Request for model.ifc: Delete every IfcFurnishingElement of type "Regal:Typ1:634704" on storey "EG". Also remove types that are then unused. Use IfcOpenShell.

First a look at what the model holds.

```python
import ifcopenshell
import ifcopenshell.util.element

model = ifcopenshell.open("model.ifc")
print(model.schema)
storey = next(s for s in model.by_type("IfcBuildingStorey") if s.Name == "EG")
furniture = [e for e in ifcopenshell.util.element.get_decomposition(storey) if e.is_a("IfcFurnishingElement")]
seen = {}
for e in furniture:
    element_type = ifcopenshell.util.element.get_type(e)
    name = element_type.Name if element_type not in (None, e) else None
    seen[name] = seen.get(name, 0) + 1
for name, count in sorted(seen.items(), key=str):
    print(count, "x", name)
```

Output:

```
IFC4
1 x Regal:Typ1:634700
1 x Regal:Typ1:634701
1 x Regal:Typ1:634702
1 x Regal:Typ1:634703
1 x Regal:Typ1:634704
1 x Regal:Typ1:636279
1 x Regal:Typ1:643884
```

```python
import ifcopenshell
import ifcopenshell.api.root
import ifcopenshell.util.element

model = ifcopenshell.open("model.ifc")

storey = next(s for s in model.by_type("IfcBuildingStorey") if s.Name == "EG")
furniture = [e for e in ifcopenshell.util.element.get_decomposition(storey) if e.is_a("IfcFurnishingElement")]
targets = [e for e in furniture if (t := ifcopenshell.util.element.get_type(e)) not in (None, e) and t.Name == "Regal:Typ1:634704"]
types = {ifcopenshell.util.element.get_type(e) for e in targets} - {None, *targets}

for e in targets:
    ifcopenshell.api.root.remove_product(model, product=e)
print(len(targets), "removed")

unused = [t for t in types if not ifcopenshell.util.element.get_types(t)]
for t in unused:
    ifcopenshell.api.root.remove_product(model, product=t)
print(len(unused), "unused types removed")

model.write("model_edited.ifc")
```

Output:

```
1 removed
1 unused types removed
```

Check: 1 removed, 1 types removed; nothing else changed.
